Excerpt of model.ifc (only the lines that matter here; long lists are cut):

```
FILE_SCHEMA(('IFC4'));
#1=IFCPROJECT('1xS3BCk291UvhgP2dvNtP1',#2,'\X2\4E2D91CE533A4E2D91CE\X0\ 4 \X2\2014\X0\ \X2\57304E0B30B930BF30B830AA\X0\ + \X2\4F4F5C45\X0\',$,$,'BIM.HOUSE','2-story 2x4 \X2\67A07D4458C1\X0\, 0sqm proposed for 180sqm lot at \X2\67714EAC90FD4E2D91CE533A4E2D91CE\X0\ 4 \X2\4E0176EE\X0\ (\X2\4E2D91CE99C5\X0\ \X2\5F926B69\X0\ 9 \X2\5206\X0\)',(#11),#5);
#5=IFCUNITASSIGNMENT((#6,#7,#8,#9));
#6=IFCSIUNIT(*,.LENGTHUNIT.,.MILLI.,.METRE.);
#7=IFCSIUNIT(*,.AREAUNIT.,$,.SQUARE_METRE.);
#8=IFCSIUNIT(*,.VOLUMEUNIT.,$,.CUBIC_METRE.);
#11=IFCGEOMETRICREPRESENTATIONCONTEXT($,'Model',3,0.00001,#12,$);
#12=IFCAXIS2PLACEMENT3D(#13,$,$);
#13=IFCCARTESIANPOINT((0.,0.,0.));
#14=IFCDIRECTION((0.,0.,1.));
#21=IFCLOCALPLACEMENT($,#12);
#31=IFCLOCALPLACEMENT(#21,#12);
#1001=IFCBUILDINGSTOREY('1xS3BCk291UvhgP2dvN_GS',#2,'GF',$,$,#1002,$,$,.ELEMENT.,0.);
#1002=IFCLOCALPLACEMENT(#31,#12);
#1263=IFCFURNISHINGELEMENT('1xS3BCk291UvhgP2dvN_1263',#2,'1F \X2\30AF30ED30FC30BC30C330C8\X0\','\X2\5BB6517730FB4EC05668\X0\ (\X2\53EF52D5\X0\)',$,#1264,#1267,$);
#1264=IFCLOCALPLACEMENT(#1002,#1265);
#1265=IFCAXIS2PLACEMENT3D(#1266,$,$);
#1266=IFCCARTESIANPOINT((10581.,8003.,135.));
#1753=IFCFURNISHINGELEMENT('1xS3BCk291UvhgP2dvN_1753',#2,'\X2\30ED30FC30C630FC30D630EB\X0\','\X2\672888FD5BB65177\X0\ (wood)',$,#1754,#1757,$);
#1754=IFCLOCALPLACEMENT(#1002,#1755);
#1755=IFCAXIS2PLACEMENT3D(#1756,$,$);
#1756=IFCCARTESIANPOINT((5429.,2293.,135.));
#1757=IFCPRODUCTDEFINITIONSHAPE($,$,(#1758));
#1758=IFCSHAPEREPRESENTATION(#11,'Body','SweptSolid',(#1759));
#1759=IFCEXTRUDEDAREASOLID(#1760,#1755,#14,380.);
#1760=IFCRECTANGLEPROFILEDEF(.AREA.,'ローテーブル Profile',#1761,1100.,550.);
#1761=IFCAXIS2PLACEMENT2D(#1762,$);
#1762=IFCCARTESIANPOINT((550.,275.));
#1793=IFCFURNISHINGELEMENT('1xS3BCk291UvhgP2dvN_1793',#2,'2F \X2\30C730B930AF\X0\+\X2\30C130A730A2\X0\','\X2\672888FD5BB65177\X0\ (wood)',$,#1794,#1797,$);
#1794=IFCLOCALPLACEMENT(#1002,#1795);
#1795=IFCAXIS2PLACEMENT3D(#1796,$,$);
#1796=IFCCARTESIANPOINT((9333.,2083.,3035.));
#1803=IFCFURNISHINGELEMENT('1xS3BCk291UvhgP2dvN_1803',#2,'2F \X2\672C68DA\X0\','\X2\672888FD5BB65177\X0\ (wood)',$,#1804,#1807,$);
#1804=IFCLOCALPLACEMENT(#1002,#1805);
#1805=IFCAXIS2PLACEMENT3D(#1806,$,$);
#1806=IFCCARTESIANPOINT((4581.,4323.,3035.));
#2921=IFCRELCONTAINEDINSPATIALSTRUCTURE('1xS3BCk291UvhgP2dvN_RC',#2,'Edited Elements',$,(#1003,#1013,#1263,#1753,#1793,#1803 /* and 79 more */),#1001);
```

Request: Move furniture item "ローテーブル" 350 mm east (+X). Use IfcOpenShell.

```python
import ifcopenshell
import ifcopenshell.api.geometry
import ifcopenshell.util.placement
import ifcopenshell.util.unit

model = ifcopenshell.open("model.ifc")
unit_scale = ifcopenshell.util.unit.calculate_unit_scale(model)

item = model.by_guid("1xS3BCk291UvhgP2dvN_1753")
matrix = ifcopenshell.util.placement.get_local_placement(item.ObjectPlacement)
matrix[0, 3] += 0.35 / unit_scale
ifcopenshell.api.geometry.edit_object_placement(model, product=item, matrix=matrix, is_si=False)

print(ifcopenshell.util.placement.get_local_placement(item.ObjectPlacement).round(3) + 0.0)

model.write("model_v2.ifc")
```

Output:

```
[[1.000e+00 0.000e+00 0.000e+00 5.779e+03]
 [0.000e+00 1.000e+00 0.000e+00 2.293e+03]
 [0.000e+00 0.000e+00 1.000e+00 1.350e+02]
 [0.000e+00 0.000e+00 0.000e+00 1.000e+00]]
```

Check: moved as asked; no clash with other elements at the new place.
